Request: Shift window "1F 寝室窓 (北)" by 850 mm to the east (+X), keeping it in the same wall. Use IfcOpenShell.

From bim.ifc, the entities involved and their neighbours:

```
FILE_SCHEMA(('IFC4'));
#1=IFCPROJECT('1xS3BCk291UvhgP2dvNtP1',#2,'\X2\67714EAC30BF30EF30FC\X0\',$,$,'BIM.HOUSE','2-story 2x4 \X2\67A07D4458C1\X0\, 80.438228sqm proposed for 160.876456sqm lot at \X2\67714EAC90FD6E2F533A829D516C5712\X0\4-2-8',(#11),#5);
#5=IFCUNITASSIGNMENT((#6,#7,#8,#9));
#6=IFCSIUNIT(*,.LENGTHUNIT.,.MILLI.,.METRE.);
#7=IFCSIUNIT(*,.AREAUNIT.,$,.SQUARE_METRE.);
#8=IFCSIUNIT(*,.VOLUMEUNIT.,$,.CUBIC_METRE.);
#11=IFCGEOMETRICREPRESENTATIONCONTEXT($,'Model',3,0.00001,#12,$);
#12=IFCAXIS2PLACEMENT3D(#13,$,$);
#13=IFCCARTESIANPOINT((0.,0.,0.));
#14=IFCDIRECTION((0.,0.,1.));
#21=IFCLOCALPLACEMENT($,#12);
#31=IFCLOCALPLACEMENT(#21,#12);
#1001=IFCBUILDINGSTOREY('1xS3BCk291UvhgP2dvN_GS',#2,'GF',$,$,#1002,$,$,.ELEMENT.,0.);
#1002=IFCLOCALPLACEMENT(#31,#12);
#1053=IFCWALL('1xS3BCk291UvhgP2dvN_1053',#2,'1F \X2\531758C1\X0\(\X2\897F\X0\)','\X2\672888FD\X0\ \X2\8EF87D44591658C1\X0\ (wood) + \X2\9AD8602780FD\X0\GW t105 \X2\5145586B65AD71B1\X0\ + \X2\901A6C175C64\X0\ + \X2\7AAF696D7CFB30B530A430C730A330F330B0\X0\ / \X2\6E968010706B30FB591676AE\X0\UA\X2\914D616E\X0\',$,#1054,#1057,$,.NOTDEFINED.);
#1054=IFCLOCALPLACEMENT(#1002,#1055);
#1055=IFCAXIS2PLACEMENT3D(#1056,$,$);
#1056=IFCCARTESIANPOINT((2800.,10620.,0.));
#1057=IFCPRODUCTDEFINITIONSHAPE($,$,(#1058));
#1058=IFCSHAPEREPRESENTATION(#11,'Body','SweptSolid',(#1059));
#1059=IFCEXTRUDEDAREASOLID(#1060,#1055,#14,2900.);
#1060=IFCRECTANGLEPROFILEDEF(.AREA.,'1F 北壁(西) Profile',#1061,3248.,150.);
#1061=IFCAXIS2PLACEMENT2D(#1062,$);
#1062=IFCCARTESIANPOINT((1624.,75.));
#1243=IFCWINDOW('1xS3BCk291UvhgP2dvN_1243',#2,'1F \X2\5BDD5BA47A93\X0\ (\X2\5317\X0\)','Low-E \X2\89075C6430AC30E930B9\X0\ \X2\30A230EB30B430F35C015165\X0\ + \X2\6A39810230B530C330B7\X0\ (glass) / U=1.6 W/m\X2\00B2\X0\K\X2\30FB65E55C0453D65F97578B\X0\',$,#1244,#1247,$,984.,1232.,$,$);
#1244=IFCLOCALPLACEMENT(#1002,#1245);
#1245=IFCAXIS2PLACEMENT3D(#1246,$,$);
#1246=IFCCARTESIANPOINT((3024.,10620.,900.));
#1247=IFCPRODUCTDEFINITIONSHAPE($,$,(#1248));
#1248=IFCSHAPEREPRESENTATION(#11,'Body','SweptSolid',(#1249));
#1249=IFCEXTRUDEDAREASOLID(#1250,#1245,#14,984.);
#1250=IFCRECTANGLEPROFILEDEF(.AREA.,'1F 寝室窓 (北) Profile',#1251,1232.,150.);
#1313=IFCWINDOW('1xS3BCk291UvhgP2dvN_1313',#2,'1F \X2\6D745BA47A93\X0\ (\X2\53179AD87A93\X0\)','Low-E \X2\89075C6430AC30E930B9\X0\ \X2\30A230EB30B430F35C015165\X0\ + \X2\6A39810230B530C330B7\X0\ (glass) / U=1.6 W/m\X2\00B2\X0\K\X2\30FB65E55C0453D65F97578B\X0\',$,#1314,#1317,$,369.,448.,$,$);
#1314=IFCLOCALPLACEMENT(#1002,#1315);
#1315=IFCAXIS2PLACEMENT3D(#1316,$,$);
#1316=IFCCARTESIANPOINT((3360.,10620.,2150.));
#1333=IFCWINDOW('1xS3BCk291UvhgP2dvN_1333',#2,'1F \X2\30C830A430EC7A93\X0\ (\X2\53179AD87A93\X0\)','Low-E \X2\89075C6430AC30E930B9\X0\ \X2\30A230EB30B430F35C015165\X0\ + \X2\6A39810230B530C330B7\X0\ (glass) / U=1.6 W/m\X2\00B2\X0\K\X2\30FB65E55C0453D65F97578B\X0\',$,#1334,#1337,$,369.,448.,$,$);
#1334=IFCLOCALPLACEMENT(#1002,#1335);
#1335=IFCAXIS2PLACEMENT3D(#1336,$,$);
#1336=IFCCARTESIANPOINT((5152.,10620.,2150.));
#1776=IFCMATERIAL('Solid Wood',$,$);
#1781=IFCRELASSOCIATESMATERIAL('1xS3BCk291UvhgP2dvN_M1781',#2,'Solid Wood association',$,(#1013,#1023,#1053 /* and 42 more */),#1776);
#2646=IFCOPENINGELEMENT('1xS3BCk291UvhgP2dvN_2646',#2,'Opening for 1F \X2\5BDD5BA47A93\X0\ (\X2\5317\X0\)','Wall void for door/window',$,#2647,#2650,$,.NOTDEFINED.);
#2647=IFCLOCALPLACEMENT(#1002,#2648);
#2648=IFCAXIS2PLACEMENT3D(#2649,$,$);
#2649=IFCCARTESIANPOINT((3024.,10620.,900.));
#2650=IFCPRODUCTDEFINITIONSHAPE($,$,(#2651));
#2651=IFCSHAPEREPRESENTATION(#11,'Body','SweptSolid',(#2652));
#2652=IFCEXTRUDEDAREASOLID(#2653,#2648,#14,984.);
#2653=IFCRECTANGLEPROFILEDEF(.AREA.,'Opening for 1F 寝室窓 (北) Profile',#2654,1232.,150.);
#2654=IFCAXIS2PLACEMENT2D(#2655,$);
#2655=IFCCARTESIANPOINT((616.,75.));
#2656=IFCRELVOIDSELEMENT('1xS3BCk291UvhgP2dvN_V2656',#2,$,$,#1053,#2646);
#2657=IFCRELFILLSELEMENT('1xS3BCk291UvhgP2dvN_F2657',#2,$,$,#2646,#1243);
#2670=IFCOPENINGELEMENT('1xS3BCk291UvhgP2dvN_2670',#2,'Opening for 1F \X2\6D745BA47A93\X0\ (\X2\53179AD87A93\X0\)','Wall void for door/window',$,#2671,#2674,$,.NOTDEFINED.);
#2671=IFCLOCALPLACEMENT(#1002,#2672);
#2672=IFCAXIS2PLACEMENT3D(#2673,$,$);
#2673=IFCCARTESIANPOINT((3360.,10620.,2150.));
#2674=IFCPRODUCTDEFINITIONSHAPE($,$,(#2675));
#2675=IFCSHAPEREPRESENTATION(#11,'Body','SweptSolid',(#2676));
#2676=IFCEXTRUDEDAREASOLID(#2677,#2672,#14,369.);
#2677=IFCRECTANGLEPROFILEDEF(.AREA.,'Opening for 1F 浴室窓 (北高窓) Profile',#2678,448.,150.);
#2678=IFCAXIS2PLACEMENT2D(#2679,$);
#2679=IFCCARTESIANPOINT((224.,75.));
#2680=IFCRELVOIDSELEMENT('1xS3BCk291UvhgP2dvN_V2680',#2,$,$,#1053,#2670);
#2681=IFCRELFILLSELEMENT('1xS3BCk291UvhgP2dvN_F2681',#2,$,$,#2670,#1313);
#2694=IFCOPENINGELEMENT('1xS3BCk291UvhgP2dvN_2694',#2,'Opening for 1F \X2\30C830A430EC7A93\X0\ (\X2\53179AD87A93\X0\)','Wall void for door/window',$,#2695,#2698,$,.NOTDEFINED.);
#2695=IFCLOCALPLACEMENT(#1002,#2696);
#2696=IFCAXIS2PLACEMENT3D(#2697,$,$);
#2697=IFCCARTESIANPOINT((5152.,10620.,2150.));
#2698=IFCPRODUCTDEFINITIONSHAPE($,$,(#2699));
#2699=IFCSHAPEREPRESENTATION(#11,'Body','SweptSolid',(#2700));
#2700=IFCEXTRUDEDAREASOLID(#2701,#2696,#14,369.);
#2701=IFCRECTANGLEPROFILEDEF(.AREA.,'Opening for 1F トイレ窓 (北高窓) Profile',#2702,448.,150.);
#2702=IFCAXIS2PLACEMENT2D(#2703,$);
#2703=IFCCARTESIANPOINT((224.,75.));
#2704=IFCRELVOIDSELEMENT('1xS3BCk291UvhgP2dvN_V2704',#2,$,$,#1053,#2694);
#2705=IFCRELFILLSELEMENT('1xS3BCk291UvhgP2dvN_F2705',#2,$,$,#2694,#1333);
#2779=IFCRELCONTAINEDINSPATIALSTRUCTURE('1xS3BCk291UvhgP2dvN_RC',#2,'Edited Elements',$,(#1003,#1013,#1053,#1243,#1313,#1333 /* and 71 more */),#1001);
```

```python
import ifcopenshell
import ifcopenshell.api.geometry
import ifcopenshell.util.placement

model = ifcopenshell.open("bim.ifc")

window = model.by_guid("1xS3BCk291UvhgP2dvN_1243")
opening = window.FillsVoids[0].RelatingOpeningElement
wall = opening.VoidsElements[0].RelatingBuildingElement

wall_matrix = ifcopenshell.util.placement.get_local_placement(wall.ObjectPlacement)
shift = wall_matrix[:3, 0] * 850.0
before = ifcopenshell.util.placement.get_local_placement(window.ObjectPlacement)[:3, 3].copy()

# The window is not placed relative to its opening, so move both.
for product in (opening, window):
    matrix = ifcopenshell.util.placement.get_local_placement(product.ObjectPlacement)
    matrix[:3, 3] += shift
    ifcopenshell.api.geometry.edit_object_placement(model, product=product, matrix=matrix, is_si=False)

after = ifcopenshell.util.placement.get_local_placement(window.ObjectPlacement)[:3, 3]
print("window moved by", (after - before).round(3) + 0.0)

model.write("bim_rev.ifc")
```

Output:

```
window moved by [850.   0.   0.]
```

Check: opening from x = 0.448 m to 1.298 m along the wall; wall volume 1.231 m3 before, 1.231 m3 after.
